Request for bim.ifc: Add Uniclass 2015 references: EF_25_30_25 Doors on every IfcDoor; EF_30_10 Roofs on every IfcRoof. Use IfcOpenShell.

First a look at what the model holds.

```python
import ifcopenshell

model = ifcopenshell.open("bim.ifc")
print(model.schema)
print("classifications:", [c.Name for c in model.by_type("IfcClassification")])
for ifc_class in ("IfcDoor", "IfcRoof", "IfcStair", "IfcWall", "IfcWindow"):
    print(ifc_class, len(model.by_type(ifc_class)))
```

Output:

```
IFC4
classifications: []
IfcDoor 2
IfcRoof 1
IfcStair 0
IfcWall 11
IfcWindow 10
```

```python
import ifcopenshell
import ifcopenshell.api.classification

model = ifcopenshell.open("bim.ifc")

system = ifcopenshell.api.classification.add_classification(model, classification="Uniclass 2015")

codes = {
    "IfcDoor": ("EF_25_30_25", "Doors"),
    "IfcRoof": ("EF_30_10", "Roofs"),
}
for ifc_class, (code, name) in codes.items():
    products = model.by_type(ifc_class)
    ifcopenshell.api.classification.add_reference(
        model, products=products, classification=system, identification=code, name=name
    )
    print(code, len(products))

model.write("bim_rev.ifc")
```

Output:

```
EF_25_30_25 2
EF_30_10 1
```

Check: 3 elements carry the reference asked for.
